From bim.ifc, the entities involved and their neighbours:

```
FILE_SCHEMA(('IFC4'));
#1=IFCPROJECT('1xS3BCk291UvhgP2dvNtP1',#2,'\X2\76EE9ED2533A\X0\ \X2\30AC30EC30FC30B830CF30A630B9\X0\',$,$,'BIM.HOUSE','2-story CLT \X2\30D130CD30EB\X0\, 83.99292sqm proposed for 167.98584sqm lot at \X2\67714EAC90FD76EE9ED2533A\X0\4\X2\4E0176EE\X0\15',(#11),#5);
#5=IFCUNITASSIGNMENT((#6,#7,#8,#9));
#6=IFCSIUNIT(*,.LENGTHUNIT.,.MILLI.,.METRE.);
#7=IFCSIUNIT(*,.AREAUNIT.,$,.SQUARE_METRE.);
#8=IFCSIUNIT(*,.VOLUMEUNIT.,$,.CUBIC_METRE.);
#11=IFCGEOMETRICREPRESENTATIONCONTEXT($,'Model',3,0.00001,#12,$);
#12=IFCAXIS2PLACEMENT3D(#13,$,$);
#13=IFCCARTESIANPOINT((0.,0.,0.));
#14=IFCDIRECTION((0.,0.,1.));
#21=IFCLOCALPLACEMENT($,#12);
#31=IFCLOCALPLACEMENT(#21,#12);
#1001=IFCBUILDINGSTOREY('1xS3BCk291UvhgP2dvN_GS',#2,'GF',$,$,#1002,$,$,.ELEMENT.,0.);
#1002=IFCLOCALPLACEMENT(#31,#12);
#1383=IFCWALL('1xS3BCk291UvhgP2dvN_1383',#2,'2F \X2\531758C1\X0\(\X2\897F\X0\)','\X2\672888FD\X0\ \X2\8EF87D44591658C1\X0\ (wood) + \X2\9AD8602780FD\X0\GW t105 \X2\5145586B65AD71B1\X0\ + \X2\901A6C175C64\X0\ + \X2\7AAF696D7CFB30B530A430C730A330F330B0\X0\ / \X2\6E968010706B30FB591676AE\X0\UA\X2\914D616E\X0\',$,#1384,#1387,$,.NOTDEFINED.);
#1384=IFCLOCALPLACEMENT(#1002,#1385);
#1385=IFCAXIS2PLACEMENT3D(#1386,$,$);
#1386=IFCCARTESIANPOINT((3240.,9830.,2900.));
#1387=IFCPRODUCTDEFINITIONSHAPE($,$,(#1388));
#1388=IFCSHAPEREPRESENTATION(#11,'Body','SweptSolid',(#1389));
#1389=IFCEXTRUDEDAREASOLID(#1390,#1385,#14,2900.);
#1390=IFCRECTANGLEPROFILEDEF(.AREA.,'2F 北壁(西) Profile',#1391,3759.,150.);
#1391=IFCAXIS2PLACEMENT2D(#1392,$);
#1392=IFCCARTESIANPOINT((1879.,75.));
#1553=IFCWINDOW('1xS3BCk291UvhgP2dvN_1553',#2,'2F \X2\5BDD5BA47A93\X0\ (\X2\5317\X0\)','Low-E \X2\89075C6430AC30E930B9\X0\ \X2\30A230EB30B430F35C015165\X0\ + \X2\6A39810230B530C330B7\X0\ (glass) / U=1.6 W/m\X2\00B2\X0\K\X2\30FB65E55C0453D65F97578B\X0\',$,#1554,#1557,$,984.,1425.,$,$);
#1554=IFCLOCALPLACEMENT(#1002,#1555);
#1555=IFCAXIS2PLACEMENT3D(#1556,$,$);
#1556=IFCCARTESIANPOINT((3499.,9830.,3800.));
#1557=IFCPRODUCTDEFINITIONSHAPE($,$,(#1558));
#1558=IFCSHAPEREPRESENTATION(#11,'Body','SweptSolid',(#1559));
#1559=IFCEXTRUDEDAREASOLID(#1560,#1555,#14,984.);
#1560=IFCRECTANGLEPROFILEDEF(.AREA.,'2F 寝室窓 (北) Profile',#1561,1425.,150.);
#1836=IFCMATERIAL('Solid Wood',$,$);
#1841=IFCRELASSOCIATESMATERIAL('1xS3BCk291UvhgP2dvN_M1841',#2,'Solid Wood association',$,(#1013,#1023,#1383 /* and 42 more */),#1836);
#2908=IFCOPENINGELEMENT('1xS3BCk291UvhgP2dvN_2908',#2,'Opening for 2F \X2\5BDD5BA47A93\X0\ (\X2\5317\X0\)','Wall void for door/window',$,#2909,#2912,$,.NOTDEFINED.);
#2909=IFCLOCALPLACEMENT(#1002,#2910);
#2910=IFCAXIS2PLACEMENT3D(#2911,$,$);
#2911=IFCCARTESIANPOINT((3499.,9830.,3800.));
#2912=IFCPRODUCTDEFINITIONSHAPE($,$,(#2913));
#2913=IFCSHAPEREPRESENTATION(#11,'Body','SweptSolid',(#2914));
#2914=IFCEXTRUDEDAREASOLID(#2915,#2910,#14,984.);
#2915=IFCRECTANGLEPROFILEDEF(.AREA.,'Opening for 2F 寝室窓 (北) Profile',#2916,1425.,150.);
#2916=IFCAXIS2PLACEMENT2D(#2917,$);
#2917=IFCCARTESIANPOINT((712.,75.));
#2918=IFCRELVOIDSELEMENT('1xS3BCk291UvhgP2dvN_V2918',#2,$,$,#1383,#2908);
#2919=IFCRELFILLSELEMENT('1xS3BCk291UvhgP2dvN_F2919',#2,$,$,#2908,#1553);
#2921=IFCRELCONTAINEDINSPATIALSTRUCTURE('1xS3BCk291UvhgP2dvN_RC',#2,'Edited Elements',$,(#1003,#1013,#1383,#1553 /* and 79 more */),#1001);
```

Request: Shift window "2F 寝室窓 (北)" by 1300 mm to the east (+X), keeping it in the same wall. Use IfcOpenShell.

```python
import ifcopenshell
import ifcopenshell.api.geometry
import ifcopenshell.util.placement
import ifcopenshell.util.unit

model = ifcopenshell.open("bim.ifc")
unit_scale = ifcopenshell.util.unit.calculate_unit_scale(model)

window = model.by_id(1553)
opening = window.FillsVoids[0].RelatingOpeningElement
wall = opening.VoidsElements[0].RelatingBuildingElement

wall_matrix = ifcopenshell.util.placement.get_local_placement(wall.ObjectPlacement)
shift = wall_matrix[:3, 0] * 1.3 / unit_scale
before = ifcopenshell.util.placement.get_local_placement(window.ObjectPlacement)[:3, 3].copy()

# The window is not placed relative to its opening, so move both.
for product in (opening, window):
    matrix = ifcopenshell.util.placement.get_local_placement(product.ObjectPlacement)
    matrix[:3, 3] += shift
    ifcopenshell.api.geometry.edit_object_placement(model, product=product, matrix=matrix, is_si=False)

after = ifcopenshell.util.placement.get_local_placement(window.ObjectPlacement)[:3, 3]
print("window moved by", (after - before).round(3) + 0.0)

model.write("bim_v2.ifc")
```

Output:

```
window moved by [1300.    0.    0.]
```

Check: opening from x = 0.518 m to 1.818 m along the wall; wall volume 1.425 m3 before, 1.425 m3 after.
